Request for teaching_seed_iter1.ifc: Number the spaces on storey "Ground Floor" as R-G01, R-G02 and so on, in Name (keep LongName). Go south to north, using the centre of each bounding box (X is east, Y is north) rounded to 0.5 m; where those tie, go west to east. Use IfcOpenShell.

First a look at what the model holds.

```python
import ifcopenshell
import ifcopenshell.util.element
import ifcopenshell.util.placement

model = ifcopenshell.open("teaching_seed_iter1.ifc")
print(model.schema)
storey = next(s for s in model.by_type("IfcBuildingStorey") if s.Name == "Ground Floor")
spaces = [e for e in ifcopenshell.util.element.get_decomposition(storey) if e.is_a("IfcSpace")]
for e in sorted(spaces, key=lambda e: e.id()):
    origin = ifcopenshell.util.placement.get_local_placement(e.ObjectPlacement)[:3, 3]
    print(e.id(), e.Name, e.LongName, origin.round(2) + 0.0, sep=" | ")
```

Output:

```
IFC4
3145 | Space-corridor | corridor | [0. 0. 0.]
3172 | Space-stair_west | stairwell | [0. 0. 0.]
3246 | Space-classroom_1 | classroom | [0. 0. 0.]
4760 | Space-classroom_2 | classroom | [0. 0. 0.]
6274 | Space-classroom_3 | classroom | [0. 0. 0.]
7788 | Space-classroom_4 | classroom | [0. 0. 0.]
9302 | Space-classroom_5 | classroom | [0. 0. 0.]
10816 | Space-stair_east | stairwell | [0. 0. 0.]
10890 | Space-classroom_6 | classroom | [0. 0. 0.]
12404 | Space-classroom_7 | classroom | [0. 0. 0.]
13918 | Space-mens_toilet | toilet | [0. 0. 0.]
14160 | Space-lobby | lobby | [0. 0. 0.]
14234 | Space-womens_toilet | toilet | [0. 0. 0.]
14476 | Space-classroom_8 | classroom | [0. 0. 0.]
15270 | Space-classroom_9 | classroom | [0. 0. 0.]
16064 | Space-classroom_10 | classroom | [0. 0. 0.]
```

```python
import ifcopenshell
import ifcopenshell.geom
import ifcopenshell.util.element
import ifcopenshell.util.shape

model = ifcopenshell.open("teaching_seed_iter1.ifc")
settings = ifcopenshell.geom.settings()
settings.set("use-world-coords", True)


def centre(element):
    shape = ifcopenshell.geom.create_shape(settings, element)
    return ifcopenshell.util.shape.get_bbox_centroid(shape.geometry)


storey = next(s for s in model.by_type("IfcBuildingStorey") if s.Name == "Ground Floor")
spaces = [e for e in ifcopenshell.util.element.get_decomposition(storey) if e.is_a("IfcSpace")]

# Insertion points can sit at a corner or the storey origin, so sort by the geometry (in metres).
centres = {e: centre(e) for e in spaces}
spaces.sort(key=lambda e: (round(centres[e][1] / 0.5), centres[e][0]))

for i, e in enumerate(spaces, start=1):
    number = f"R-G{i:02d}"
    e.Name = number
    print(e.id(), number)

model.write("teaching_seed_iter1_v2.ifc")
```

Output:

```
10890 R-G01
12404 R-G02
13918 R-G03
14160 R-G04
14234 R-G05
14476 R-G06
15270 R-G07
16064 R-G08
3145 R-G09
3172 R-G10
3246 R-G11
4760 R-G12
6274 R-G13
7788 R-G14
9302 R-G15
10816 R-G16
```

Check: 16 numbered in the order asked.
